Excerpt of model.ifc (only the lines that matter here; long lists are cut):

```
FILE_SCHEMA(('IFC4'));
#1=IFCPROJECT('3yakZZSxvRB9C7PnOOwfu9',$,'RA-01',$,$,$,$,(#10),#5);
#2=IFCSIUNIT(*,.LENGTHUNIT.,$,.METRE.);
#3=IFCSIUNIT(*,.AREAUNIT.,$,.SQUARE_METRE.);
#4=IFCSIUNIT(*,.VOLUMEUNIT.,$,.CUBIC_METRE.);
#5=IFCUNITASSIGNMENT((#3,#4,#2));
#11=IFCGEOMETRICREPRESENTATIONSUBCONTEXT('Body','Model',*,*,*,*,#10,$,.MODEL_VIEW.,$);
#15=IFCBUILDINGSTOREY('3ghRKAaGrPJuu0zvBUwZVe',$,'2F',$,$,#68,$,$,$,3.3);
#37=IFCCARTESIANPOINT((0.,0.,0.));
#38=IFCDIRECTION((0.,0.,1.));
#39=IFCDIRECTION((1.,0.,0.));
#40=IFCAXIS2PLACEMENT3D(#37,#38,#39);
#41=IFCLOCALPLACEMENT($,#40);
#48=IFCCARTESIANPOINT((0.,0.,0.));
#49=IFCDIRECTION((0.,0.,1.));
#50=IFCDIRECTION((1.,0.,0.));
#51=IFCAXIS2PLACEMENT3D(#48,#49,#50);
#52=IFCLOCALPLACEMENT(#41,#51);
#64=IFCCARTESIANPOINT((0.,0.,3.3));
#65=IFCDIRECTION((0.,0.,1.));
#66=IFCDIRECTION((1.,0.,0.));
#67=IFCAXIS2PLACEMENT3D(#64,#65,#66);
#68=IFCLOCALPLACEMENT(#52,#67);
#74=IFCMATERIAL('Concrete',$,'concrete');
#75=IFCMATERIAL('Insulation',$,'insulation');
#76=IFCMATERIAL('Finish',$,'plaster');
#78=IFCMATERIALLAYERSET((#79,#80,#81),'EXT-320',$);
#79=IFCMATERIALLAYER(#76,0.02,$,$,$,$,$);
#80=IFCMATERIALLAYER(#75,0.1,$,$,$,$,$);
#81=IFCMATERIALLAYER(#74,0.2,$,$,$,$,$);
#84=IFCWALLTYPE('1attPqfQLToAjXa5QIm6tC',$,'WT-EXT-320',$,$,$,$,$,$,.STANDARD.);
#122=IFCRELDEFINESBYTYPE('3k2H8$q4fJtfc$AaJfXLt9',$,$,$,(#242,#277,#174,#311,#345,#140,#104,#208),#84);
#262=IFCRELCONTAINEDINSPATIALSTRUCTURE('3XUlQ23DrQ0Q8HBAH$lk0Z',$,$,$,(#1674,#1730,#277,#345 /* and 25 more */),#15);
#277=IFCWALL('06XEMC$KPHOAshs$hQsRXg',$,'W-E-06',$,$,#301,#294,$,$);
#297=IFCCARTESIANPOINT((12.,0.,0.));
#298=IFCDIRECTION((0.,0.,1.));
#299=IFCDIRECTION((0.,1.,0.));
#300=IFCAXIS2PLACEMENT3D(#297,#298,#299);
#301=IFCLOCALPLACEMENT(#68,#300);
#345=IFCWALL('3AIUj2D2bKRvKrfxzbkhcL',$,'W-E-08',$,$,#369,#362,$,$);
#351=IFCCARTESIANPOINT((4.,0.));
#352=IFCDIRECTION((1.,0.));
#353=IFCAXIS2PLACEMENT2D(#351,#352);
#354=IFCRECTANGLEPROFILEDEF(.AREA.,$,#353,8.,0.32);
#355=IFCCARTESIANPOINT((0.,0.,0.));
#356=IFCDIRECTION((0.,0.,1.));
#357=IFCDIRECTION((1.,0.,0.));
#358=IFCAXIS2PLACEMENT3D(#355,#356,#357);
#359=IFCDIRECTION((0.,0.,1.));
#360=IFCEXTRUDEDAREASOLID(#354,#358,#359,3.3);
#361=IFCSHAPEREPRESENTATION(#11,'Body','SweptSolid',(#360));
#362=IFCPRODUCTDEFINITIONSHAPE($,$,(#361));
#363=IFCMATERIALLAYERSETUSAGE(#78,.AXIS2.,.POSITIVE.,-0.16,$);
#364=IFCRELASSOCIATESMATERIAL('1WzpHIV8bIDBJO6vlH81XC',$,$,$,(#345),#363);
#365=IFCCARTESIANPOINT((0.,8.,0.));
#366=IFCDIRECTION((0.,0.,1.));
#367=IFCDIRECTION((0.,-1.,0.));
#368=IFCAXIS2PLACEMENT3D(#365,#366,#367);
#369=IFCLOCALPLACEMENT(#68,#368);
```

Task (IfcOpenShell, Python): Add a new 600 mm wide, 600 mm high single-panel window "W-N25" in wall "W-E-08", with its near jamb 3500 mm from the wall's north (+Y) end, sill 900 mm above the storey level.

```python
import numpy as np
import ifcopenshell
import ifcopenshell.api.feature
import ifcopenshell.api.geometry
import ifcopenshell.api.root
import ifcopenshell.api.spatial
import ifcopenshell.geom
import ifcopenshell.util.element
import ifcopenshell.util.placement
import ifcopenshell.util.representation
import ifcopenshell.util.shape
import ifcopenshell.util.unit

model = ifcopenshell.open("model.ifc")
unit_scale = ifcopenshell.util.unit.calculate_unit_scale(model)
settings = ifcopenshell.geom.settings()


def volume(element):
    """Net volume in cubic metres, openings subtracted."""
    shape = ifcopenshell.geom.create_shape(settings, element)
    return ifcopenshell.util.shape.get_volume(shape.geometry)


wall = model.by_guid("3AIUj2D2bKRvKrfxzbkhcL")
storey = ifcopenshell.util.element.get_container(wall, ifc_class="IfcBuildingStorey")
context = ifcopenshell.util.representation.get_context(model, "Model", "Body", "MODEL_VIEW")
before = volume(wall)

width, height, from_end, sill = 0.6, 0.6, 3.5, 0.9  # metres

# The wall runs along its own X axis, and the end named is its -X end.
wall_shape = ifcopenshell.geom.create_shape(settings, wall)
x, y, z = ifcopenshell.util.shape.get_vertices(wall_shape.geometry).T
start = x.min() + from_end
face, thickness = float(y.min()), float(y.max() - y.min())
wall_matrix = ifcopenshell.util.placement.get_local_placement(wall.ObjectPlacement)
level = ifcopenshell.util.placement.get_local_placement(storey.ObjectPlacement)[2, 3]


def in_wall(x, y):
    """Placement at x, y metres in the wall's axes, at sill height."""
    matrix = wall_matrix.copy()
    matrix[:, 3] = wall_matrix @ np.array([x / unit_scale, y / unit_scale, 0.0, 1.0])
    matrix[2, 3] = level + sill / unit_scale
    return matrix


# Opening: a box that overshoots both wall faces by 50 mm.
opening = ifcopenshell.api.root.create_entity(model, ifc_class="IfcOpeningElement", predefined_type="OPENING")
box = ifcopenshell.api.geometry.add_wall_representation(
    model, context=context, length=width, height=height, thickness=thickness + 0.1
)
ifcopenshell.api.geometry.assign_representation(model, product=opening, representation=box)
ifcopenshell.api.geometry.edit_object_placement(model, product=opening, matrix=in_wall(start, face - 0.05), is_si=False)
ifcopenshell.api.feature.add_feature(model, feature=opening, element=wall)

window = ifcopenshell.api.root.create_entity(model, ifc_class="IfcWindow", name="W-N25", predefined_type="WINDOW")
window.OverallWidth, window.OverallHeight = width / unit_scale, height / unit_scale
window.PartitioningType = "SINGLE_PANEL"
body = ifcopenshell.api.geometry.add_window_representation(
    model,
    context=context,
    overall_width=window.OverallWidth,
    overall_height=window.OverallHeight,
    partition_type="SINGLE_PANEL",
)
ifcopenshell.api.geometry.assign_representation(model, product=window, representation=body)
ifcopenshell.api.spatial.assign_container(model, products=[window], relating_structure=storey)
ifcopenshell.api.feature.add_filling(model, opening=opening, element=window)

# Centre the window in the wall's thickness.
ifcopenshell.api.geometry.edit_object_placement(model, product=window, matrix=in_wall(start, face), is_si=False)
window_shape = ifcopenshell.geom.create_shape(settings, window)
depth = ifcopenshell.util.shape.get_vertices(window_shape.geometry)[:, 1]
offset = face + thickness / 2 - (depth.min() + depth.max()) / 2
ifcopenshell.api.geometry.edit_object_placement(model, product=window, matrix=in_wall(start, offset), is_si=False)

after = volume(wall)

print(f"wall volume {before:.3f} -> {after:.3f} m3")

model.write("model_v2.ifc")
```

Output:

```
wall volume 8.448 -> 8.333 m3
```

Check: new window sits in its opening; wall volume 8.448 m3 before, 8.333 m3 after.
